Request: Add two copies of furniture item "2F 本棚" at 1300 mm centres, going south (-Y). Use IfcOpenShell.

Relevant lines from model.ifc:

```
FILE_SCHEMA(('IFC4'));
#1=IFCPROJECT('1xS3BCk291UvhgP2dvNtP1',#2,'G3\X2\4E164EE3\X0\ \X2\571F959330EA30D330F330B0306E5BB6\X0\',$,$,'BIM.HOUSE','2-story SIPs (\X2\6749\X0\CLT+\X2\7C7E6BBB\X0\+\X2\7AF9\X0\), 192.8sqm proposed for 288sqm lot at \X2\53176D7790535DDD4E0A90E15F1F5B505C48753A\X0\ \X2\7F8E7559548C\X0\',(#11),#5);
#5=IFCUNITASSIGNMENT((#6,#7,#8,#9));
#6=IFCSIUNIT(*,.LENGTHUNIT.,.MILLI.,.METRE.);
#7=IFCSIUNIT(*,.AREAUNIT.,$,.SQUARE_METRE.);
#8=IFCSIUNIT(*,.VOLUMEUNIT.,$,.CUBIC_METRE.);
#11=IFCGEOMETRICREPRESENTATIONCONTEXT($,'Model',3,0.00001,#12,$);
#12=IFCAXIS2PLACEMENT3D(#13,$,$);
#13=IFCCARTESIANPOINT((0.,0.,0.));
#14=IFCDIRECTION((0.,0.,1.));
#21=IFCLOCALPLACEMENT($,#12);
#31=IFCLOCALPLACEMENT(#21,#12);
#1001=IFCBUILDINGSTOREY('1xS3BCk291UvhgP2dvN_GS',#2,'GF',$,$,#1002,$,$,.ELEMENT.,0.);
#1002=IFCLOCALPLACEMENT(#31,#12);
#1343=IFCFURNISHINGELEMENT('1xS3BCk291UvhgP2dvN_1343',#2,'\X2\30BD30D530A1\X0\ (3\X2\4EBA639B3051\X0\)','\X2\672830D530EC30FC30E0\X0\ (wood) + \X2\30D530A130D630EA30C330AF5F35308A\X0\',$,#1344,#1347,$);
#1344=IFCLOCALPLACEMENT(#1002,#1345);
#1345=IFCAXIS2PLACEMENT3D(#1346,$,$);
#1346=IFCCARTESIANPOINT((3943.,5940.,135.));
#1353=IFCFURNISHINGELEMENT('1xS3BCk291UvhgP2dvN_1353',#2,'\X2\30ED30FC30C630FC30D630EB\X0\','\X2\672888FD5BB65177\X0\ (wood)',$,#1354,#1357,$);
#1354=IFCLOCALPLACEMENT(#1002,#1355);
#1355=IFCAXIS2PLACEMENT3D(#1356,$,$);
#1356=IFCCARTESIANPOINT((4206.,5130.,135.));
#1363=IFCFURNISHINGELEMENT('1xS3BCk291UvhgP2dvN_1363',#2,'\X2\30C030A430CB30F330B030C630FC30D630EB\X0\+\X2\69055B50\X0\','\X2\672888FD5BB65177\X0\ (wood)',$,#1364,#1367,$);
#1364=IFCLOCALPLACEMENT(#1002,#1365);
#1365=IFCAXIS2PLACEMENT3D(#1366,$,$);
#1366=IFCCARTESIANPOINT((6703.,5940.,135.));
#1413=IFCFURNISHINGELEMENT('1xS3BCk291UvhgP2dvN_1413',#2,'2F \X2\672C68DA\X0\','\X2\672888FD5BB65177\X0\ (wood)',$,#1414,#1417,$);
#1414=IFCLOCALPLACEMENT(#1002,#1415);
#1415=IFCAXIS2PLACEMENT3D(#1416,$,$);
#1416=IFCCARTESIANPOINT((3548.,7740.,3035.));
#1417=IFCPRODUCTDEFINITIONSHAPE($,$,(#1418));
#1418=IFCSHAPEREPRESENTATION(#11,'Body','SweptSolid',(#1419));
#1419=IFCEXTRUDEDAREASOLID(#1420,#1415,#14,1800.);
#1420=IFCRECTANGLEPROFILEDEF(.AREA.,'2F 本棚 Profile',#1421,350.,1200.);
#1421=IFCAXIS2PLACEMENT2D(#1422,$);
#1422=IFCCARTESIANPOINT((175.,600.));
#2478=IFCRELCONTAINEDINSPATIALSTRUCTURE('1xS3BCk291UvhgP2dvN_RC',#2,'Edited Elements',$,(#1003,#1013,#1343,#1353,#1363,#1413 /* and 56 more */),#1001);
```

```python
import numpy as np
import ifcopenshell
import ifcopenshell.api.geometry
import ifcopenshell.api.root
import ifcopenshell.util.element
import ifcopenshell.util.placement
import ifcopenshell.util.unit

model = ifcopenshell.open("model.ifc")
unit_scale = ifcopenshell.util.unit.calculate_unit_scale(model)


def reuse_history(source, copy):
    """copy_class also copies each property set's owner history, people and application; keep the originals."""
    for rel in copy.IsDefinedBy:
        if rel.is_a("IfcRelDefinesByProperties") and (history := rel.RelatingPropertyDefinition.OwnerHistory):
            rel.RelatingPropertyDefinition.OwnerHistory = source.OwnerHistory
            ifcopenshell.util.element.remove_deep2(model, history)


source = model.by_id(1413)
base = ifcopenshell.util.placement.get_local_placement(source.ObjectPlacement)
step = np.array([0.0, -1.0, 0.0]) * 1.3 / unit_scale

for i in range(1, 3):
    copy = ifcopenshell.api.root.copy_class(model, product=source)
    copy.Representation = ifcopenshell.util.element.copy_deep(
        model, source.Representation, exclude=["IfcGeometricRepresentationContext", "IfcRepresentationMap"]
    )
    reuse_history(source, copy)
    matrix = base.copy()
    matrix[:3, 3] += i * step
    print("added at", matrix[:3, 3].round(3) + 0.0)
    ifcopenshell.api.geometry.edit_object_placement(model, product=copy, matrix=matrix, is_si=False)

model.write("model_updated.ifc")
```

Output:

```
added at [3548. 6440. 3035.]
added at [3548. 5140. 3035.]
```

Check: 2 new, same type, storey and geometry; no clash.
